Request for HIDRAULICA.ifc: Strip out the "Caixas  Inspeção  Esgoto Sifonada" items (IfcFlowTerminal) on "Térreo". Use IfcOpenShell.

First a look at what the model holds.

```python
import ifcopenshell
import ifcopenshell.util.element

model = ifcopenshell.open("HIDRAULICA.ifc")
print(model.schema)
storey = next(s for s in model.by_type("IfcBuildingStorey") if s.Name == "Térreo")
terminals = [e for e in ifcopenshell.util.element.get_decomposition(storey) if e.is_a("IfcFlowTerminal")]
seen = {}
for e in terminals:
    element_type = ifcopenshell.util.element.get_type(e)
    name = element_type.Name if element_type not in (None, e) else None
    seen[name] = seen.get(name, 0) + 1
for name, count in sorted(seen.items(), key=str):
    print(count, "x", name)
```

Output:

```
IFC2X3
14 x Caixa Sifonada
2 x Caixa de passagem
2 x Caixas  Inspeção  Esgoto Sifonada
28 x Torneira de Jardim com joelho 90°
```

```python
import ifcopenshell
import ifcopenshell.api.root
import ifcopenshell.util.element

model = ifcopenshell.open("HIDRAULICA.ifc")

storey = next(s for s in model.by_type("IfcBuildingStorey") if s.Name == "Térreo")
terminals = [e for e in ifcopenshell.util.element.get_decomposition(storey) if e.is_a("IfcFlowTerminal")]
targets = [e for e in terminals if (t := ifcopenshell.util.element.get_type(e)) not in (None, e) and t.Name == "Caixas  Inspeção  Esgoto Sifonada"]

for e in targets:
    ifcopenshell.api.root.remove_product(model, product=e)
print(len(targets), "removed")

model.write("HIDRAULICA_v2.ifc")
```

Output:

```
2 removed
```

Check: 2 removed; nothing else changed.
